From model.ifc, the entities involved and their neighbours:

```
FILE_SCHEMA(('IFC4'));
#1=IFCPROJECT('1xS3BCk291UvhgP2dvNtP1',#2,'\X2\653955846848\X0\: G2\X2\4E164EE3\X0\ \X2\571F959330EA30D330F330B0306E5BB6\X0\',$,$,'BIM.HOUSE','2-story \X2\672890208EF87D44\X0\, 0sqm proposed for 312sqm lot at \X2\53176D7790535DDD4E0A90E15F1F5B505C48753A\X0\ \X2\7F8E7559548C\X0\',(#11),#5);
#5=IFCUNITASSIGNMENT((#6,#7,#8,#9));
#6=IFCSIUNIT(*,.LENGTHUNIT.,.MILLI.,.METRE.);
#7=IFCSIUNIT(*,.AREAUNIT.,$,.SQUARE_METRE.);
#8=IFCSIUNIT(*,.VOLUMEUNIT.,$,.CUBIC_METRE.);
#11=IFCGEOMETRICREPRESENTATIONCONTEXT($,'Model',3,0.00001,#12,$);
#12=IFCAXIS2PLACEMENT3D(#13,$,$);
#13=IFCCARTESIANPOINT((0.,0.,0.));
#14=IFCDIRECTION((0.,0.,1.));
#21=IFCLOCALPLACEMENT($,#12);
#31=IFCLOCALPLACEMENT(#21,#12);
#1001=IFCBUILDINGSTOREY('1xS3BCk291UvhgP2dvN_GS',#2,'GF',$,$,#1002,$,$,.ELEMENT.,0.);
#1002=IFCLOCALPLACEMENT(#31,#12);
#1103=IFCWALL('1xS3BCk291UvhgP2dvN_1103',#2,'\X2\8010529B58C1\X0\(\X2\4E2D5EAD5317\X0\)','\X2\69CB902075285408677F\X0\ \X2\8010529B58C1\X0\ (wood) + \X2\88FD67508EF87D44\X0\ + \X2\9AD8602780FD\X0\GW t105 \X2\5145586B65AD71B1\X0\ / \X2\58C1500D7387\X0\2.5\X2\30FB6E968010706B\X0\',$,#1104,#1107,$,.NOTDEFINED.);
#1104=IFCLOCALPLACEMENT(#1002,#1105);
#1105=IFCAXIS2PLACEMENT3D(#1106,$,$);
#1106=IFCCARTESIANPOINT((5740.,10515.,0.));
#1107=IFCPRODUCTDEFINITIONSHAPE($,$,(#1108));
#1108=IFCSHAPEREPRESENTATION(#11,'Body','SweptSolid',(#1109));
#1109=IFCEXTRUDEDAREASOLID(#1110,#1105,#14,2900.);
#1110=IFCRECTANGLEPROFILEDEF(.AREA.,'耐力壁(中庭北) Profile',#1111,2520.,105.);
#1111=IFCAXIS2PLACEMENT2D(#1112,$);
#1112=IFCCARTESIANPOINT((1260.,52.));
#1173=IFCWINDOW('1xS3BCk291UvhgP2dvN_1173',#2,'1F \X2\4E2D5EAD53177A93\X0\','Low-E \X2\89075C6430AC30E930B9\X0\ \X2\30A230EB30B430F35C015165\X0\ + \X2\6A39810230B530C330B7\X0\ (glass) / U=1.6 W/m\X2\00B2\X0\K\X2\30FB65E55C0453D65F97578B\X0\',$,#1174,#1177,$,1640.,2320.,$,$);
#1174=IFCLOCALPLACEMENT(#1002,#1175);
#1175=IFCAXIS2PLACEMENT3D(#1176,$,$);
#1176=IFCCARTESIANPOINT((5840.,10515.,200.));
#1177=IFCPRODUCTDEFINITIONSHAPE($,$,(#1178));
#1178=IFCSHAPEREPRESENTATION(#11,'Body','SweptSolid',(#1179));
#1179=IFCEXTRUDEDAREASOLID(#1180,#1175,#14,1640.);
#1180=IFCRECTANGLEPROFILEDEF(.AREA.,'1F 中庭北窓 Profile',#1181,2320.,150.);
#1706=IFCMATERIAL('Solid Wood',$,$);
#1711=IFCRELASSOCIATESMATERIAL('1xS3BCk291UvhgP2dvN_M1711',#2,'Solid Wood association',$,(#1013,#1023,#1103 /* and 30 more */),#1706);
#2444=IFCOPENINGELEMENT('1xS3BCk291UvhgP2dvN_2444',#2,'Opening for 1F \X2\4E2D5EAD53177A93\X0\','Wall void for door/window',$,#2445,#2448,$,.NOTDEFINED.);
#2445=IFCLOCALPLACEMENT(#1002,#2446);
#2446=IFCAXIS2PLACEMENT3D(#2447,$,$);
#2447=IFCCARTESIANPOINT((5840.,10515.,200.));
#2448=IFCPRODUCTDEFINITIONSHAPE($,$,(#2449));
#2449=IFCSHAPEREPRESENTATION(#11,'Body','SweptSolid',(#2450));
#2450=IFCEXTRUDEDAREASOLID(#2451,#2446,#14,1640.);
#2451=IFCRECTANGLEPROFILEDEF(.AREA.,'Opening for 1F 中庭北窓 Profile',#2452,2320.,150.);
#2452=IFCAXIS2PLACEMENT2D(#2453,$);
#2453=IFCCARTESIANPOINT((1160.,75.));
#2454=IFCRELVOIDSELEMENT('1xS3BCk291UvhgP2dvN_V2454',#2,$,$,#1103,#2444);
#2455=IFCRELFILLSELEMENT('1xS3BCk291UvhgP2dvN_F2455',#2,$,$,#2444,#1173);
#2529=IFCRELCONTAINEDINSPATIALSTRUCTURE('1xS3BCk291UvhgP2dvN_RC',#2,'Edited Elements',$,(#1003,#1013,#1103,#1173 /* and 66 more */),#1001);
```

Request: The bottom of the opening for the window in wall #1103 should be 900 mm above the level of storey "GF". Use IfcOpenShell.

```python
import numpy as np
import ifcopenshell
import ifcopenshell.api.geometry
import ifcopenshell.geom
import ifcopenshell.util.element
import ifcopenshell.util.placement
import ifcopenshell.util.shape
import ifcopenshell.util.unit

model = ifcopenshell.open("model.ifc")
unit_scale = ifcopenshell.util.unit.calculate_unit_scale(model)

window = model.by_id(1173)
opening = window.FillsVoids[0].RelatingOpeningElement
storey = ifcopenshell.util.element.get_container(window, ifc_class="IfcBuildingStorey")
level = ifcopenshell.util.placement.get_local_placement(storey.ObjectPlacement)[2, 3]

# The opening's origin need not be at the sill, so measure its lowest point.
shape = ifcopenshell.geom.create_shape(ifcopenshell.geom.settings(), opening)
bottom = ifcopenshell.util.shape.get_shape_bottom_elevation(shape, shape.geometry) / unit_scale
dz = level + 0.9 / unit_scale - bottom

shift = np.array([0.0, 0.0, dz])
# The window is not placed relative to its opening, so move both.
for product in (opening, window):
    matrix = ifcopenshell.util.placement.get_local_placement(product.ObjectPlacement)
    matrix[:3, 3] += shift
    ifcopenshell.api.geometry.edit_object_placement(model, product=product, matrix=matrix, is_si=False)

print(f"moved by {dz * unit_scale:+.3f} m")

model.write("model_edited.ifc")
```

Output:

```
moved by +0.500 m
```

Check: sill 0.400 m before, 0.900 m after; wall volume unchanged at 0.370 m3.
